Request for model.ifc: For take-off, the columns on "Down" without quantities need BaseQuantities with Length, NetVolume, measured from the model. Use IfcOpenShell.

First a look at what the model holds.

```python
import ifcopenshell
import ifcopenshell.util.element
import ifcopenshell.util.unit

model = ifcopenshell.open("model.ifc")
print(model.schema)
for unit_type in ("LENGTHUNIT", "AREAUNIT", "VOLUMEUNIT"):
    print(unit_type, ifcopenshell.util.unit.calculate_unit_scale(model, unit_type))
storey = next(s for s in model.by_type("IfcBuildingStorey") if s.Name == "Down")
columns = [e for e in ifcopenshell.util.element.get_decomposition(storey) if e.is_a("IfcColumn")]
for e in sorted(columns, key=lambda e: e.id()):
    print(e.id(), e.is_a(), e.Name, list(ifcopenshell.util.element.get_psets(e, qtos_only=True)), sep=" | ")
```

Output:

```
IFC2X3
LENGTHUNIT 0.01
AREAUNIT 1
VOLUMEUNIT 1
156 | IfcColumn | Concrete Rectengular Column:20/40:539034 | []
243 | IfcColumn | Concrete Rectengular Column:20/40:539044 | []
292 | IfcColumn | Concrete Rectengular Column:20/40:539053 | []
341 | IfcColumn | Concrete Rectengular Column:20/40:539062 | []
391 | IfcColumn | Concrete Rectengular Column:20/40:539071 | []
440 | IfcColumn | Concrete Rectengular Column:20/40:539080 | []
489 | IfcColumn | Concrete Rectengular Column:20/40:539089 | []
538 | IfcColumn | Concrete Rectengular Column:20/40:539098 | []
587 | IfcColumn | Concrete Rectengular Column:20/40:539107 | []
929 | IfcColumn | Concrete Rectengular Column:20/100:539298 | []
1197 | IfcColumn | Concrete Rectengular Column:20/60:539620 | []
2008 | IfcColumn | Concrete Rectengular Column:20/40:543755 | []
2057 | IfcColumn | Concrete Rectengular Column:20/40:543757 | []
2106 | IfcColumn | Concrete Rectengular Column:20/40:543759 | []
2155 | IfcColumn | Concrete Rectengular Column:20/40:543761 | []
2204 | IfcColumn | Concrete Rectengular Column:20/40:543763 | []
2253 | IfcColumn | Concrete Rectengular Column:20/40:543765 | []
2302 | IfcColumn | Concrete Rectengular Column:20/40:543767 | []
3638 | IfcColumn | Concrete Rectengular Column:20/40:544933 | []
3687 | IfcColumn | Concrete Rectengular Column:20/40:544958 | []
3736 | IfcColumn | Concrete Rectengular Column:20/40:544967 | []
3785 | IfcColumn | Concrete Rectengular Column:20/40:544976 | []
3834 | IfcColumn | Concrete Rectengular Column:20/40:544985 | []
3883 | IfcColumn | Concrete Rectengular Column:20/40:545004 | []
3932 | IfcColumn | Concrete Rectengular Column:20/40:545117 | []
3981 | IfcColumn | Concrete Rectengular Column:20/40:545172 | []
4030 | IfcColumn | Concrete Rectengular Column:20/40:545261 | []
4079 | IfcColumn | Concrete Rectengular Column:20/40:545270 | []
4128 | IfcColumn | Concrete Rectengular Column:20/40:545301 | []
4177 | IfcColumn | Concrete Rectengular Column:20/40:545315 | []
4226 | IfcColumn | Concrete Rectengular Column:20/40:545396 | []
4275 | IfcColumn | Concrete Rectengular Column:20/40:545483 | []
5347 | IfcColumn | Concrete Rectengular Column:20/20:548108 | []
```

```python
import ifcopenshell
import ifcopenshell.api.pset
import ifcopenshell.geom
import ifcopenshell.util.element
import ifcopenshell.util.shape
import ifcopenshell.util.unit

model = ifcopenshell.open("model.ifc")
unit_scale = ifcopenshell.util.unit.calculate_unit_scale(model)
volume_scale = ifcopenshell.util.unit.calculate_unit_scale(model, "VOLUMEUNIT")
settings = ifcopenshell.geom.settings()

storey = next(s for s in model.by_type("IfcBuildingStorey") if s.Name == "Down")
columns = [e for e in ifcopenshell.util.element.get_decomposition(storey) if e.is_a("IfcColumn")]

for e in sorted(columns, key=lambda e: e.id()):
    if ifcopenshell.util.element.get_psets(e, qtos_only=True, should_inherit=False):
        continue
    # Geometry comes back in metres, in the element's own axes.
    shape = ifcopenshell.geom.create_shape(settings, e)
    values = {
        "Length": ifcopenshell.util.shape.get_z(shape.geometry) / unit_scale,
        "NetVolume": ifcopenshell.util.shape.get_volume(shape.geometry) / volume_scale,
    }
    qto = ifcopenshell.api.pset.add_qto(model, product=e, name="BaseQuantities")
    ifcopenshell.api.pset.edit_qto(model, qto=qto, properties=values)
    print(e.id(), {k: round(v, 3) for k, v in values.items()})

model.write("model_v2.ifc")
```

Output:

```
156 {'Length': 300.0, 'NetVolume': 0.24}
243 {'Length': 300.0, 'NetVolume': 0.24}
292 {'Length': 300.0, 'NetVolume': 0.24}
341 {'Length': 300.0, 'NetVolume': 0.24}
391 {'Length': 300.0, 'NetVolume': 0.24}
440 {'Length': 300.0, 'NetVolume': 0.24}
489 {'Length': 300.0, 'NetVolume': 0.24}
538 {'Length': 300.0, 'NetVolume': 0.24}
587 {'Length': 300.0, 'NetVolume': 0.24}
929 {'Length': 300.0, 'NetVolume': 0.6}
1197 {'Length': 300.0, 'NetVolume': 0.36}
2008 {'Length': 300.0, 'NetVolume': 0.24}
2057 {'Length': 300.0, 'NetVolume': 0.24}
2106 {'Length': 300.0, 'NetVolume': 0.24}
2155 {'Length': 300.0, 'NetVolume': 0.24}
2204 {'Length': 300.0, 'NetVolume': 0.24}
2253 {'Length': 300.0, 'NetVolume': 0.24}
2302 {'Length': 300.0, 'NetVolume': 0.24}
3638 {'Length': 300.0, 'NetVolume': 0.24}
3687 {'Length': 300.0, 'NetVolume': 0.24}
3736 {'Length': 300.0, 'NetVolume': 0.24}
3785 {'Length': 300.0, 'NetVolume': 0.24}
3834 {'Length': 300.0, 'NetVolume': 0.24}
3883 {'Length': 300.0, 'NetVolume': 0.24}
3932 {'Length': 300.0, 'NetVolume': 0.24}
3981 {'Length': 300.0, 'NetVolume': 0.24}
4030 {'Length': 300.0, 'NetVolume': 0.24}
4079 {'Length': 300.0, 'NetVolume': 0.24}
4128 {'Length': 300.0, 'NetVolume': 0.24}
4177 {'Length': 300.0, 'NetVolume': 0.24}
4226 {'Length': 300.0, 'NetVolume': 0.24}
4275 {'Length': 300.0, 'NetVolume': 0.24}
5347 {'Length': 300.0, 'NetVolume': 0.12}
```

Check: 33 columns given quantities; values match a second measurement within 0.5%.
